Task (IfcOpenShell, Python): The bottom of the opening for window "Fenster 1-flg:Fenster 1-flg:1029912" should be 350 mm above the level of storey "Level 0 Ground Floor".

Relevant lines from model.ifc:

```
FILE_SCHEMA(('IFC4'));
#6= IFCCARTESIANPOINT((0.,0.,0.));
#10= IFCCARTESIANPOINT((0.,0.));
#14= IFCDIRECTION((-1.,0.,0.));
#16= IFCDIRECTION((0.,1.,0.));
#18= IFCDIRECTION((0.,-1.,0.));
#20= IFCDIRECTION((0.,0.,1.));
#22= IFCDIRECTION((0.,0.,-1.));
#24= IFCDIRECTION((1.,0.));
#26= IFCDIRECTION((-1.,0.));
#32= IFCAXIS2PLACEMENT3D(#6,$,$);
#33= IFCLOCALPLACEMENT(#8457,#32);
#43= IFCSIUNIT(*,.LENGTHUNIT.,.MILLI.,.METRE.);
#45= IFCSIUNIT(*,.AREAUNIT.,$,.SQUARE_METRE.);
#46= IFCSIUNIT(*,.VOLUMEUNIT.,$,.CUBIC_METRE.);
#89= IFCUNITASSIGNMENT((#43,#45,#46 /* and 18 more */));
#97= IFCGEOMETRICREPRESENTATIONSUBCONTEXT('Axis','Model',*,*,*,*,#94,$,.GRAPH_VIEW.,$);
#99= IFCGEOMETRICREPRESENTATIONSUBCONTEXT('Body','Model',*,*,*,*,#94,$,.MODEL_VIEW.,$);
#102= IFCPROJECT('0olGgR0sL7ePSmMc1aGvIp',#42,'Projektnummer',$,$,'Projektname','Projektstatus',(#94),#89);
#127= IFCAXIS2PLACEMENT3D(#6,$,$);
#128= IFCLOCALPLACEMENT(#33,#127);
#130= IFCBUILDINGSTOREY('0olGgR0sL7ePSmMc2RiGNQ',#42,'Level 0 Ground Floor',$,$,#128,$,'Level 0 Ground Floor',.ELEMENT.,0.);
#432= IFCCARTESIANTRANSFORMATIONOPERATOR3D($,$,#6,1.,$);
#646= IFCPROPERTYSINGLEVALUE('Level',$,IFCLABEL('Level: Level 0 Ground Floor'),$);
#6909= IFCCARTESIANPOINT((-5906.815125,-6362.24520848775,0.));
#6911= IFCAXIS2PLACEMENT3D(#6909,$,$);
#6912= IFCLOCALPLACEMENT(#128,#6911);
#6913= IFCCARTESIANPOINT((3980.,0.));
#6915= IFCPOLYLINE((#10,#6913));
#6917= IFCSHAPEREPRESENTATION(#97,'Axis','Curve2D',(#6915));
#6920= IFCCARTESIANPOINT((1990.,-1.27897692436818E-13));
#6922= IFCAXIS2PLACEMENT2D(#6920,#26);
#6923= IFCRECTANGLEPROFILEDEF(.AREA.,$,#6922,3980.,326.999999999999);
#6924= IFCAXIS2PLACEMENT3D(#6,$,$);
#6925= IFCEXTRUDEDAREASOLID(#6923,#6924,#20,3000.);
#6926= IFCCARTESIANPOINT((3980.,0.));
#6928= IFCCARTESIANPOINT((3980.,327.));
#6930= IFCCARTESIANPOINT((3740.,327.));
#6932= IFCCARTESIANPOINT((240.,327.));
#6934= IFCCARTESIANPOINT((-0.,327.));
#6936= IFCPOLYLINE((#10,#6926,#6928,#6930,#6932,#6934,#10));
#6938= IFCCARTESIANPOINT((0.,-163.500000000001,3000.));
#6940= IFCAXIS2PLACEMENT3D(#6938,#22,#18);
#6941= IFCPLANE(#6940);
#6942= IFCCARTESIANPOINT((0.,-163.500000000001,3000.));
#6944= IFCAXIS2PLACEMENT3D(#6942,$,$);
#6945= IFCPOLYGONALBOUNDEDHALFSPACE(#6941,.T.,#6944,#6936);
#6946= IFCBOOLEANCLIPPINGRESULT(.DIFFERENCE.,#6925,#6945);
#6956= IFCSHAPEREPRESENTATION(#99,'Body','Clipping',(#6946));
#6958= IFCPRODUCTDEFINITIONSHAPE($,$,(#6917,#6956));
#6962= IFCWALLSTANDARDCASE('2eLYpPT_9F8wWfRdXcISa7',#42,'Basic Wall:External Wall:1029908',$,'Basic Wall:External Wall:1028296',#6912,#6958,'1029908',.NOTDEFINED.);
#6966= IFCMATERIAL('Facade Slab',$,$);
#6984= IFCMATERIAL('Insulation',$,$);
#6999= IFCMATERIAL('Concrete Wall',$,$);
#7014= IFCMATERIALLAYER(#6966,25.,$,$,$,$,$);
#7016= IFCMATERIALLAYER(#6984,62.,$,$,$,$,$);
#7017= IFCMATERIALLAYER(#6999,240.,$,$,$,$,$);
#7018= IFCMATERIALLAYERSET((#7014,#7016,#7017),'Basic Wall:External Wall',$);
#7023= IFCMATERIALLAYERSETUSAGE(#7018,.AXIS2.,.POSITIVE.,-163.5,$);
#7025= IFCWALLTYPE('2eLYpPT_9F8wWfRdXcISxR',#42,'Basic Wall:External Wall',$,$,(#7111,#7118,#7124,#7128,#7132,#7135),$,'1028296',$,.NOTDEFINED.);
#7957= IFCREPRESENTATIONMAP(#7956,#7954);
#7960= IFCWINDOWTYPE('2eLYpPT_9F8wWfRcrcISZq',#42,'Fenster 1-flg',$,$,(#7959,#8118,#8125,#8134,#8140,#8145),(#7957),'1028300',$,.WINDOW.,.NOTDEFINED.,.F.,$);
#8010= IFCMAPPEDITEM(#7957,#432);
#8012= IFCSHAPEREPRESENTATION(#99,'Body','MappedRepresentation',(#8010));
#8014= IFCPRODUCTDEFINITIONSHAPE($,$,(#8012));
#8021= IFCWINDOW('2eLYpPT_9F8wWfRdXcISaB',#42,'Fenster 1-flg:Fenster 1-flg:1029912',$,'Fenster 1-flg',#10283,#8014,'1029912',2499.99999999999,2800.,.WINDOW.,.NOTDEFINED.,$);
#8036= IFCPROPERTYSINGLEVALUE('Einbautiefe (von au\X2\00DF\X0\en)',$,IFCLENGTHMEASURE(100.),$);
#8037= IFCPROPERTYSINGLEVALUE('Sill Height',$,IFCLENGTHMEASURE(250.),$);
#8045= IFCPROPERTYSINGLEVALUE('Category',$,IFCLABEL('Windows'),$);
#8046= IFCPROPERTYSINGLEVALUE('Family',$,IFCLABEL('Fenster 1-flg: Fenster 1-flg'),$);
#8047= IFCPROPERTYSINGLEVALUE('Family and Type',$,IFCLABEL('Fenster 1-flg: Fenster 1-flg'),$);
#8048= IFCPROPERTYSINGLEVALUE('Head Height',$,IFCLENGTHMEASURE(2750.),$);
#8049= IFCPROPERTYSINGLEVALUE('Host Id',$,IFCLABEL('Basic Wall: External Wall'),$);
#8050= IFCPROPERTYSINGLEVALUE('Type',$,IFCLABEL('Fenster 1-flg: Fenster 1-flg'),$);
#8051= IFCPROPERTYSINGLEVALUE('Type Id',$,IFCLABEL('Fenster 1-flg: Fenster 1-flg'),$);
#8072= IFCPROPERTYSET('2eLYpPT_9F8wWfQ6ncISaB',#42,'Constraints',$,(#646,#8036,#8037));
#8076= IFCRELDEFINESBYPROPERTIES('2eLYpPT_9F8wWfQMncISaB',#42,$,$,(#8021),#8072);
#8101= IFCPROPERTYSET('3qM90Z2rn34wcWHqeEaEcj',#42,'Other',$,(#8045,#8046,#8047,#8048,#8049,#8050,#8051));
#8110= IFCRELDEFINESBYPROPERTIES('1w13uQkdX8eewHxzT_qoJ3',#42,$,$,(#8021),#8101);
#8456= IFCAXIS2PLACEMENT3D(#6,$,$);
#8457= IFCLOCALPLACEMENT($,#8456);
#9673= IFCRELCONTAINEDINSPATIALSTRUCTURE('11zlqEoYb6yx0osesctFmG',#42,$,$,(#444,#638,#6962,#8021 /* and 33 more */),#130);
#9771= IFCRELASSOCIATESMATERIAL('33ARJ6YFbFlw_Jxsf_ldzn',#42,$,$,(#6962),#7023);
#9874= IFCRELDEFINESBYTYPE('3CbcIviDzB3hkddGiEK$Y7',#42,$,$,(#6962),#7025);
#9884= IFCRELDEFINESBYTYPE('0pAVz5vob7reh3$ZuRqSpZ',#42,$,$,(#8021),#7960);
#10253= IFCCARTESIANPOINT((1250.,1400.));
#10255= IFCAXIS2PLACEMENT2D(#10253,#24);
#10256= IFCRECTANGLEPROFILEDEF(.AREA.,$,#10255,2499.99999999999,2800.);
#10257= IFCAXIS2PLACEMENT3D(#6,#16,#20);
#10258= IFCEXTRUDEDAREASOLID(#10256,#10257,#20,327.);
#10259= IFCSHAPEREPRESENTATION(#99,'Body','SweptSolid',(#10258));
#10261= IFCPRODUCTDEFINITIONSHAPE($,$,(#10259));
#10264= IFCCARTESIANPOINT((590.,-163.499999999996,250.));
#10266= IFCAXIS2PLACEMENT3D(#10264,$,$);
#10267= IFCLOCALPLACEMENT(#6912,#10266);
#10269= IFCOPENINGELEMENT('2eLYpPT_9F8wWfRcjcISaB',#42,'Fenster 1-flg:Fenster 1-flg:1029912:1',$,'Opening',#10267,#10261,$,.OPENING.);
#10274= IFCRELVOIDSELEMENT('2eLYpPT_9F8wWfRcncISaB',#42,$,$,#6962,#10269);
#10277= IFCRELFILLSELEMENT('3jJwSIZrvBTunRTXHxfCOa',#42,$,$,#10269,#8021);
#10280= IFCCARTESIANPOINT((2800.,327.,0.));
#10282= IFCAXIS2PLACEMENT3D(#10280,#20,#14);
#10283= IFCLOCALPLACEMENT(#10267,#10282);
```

```python
import numpy as np
import ifcopenshell
import ifcopenshell.api.geometry
import ifcopenshell.api.pset
import ifcopenshell.geom
import ifcopenshell.util.element
import ifcopenshell.util.placement
import ifcopenshell.util.shape
import ifcopenshell.util.unit

model = ifcopenshell.open("model.ifc")
unit_scale = ifcopenshell.util.unit.calculate_unit_scale(model)

window = model.by_guid("2eLYpPT_9F8wWfRdXcISaB")
opening = window.FillsVoids[0].RelatingOpeningElement
storey = ifcopenshell.util.element.get_container(window, ifc_class="IfcBuildingStorey")
level = ifcopenshell.util.placement.get_local_placement(storey.ObjectPlacement)[2, 3]

# The opening's origin need not be at the sill, so measure its lowest point.
shape = ifcopenshell.geom.create_shape(ifcopenshell.geom.settings(), opening)
bottom = ifcopenshell.util.shape.get_shape_bottom_elevation(shape, shape.geometry) / unit_scale
dz = level + 350.0 - bottom

shift = np.array([0.0, 0.0, dz])
# The window is placed relative to its opening, so it follows when the opening moves.
matrix = ifcopenshell.util.placement.get_local_placement(opening.ObjectPlacement)
matrix[:3, 3] += shift
ifcopenshell.api.geometry.edit_object_placement(
    model, product=opening, matrix=matrix, is_si=False, should_transform_children=True
)

# Keep the stored heights in step.
pset = model.by_id(ifcopenshell.util.element.get_pset(window, "Constraints", should_inherit=False)["id"])
ifcopenshell.api.pset.edit_pset(model, pset=pset, properties={
    "Sill Height": model.create_entity("IfcLengthMeasure", ifcopenshell.util.element.get_pset(window, "Constraints", "Sill Height") + dz),
})
pset = model.by_id(ifcopenshell.util.element.get_pset(window, "Other", should_inherit=False)["id"])
ifcopenshell.api.pset.edit_pset(model, pset=pset, properties={
    "Head Height": model.create_entity("IfcLengthMeasure", ifcopenshell.util.element.get_pset(window, "Other", "Head Height") + dz),
})

print(f"moved by {dz * unit_scale:+.3f} m")

model.write("model_updated.ifc")
```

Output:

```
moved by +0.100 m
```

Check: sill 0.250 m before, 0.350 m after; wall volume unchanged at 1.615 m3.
